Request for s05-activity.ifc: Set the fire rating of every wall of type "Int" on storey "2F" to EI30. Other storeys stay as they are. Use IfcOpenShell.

First a look at what the model holds.

```python
import ifcopenshell
import ifcopenshell.util.element

model = ifcopenshell.open("s05-activity.ifc")
print(model.schema)
storey = next(s for s in model.by_type("IfcBuildingStorey") if s.Name == "2F")
walls = [e for e in ifcopenshell.util.element.get_decomposition(storey) if e.is_a("IfcWall")]
seen = {}
for e in walls:
    element_type = ifcopenshell.util.element.get_type(e)
    key = (element_type.Name if element_type != e and element_type else None, ifcopenshell.util.element.get_pset(e, "Pset_WallCommon", "FireRating"))
    seen[key] = seen.get(key, 0) + 1
for (name, value), count in sorted(seen.items(), key=str):
    print(count, "x", name, "|", value)
```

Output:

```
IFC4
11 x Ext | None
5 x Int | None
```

```python
import ifcopenshell
import ifcopenshell.api.pset
import ifcopenshell.util.element

model = ifcopenshell.open("s05-activity.ifc")

storey = next(s for s in model.by_type("IfcBuildingStorey") if s.Name == "2F")
walls = [e for e in ifcopenshell.util.element.get_decomposition(storey) if e.is_a("IfcWall")]

count = 0
for e in walls:
    element_type = ifcopenshell.util.element.get_type(e)
    if element_type in (None, e) or element_type.Name != "Int":
        continue
    # add_pset returns the element's existing set when there is one.
    pset = ifcopenshell.api.pset.add_pset(model, product=e, name="Pset_WallCommon")
    ifcopenshell.api.pset.edit_pset(model, pset=pset, properties={"FireRating": "EI30"})
    count += 1

print(count, "walls updated")

model.write("s05-activity_rev.ifc")
```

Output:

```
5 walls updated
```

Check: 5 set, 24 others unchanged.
